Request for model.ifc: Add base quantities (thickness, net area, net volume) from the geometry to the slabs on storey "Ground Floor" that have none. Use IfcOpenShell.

First a look at what the model holds.

```python
import ifcopenshell
import ifcopenshell.util.element
import ifcopenshell.util.unit

model = ifcopenshell.open("model.ifc")
print(model.schema)
for unit_type in ("LENGTHUNIT", "AREAUNIT", "VOLUMEUNIT"):
    print(unit_type, ifcopenshell.util.unit.calculate_unit_scale(model, unit_type))
storey = next(s for s in model.by_type("IfcBuildingStorey") if s.Name == "Ground Floor")
slabs = [e for e in ifcopenshell.util.element.get_decomposition(storey) if e.is_a("IfcSlab")]
for e in sorted(slabs, key=lambda e: e.id()):
    print(e.id(), e.is_a(), e.Name, list(ifcopenshell.util.element.get_psets(e, qtos_only=True)), sep=" | ")
```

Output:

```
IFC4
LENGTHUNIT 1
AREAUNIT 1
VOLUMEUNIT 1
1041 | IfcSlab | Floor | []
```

```python
import ifcopenshell
import ifcopenshell.api.pset
import ifcopenshell.geom
import ifcopenshell.util.element
import ifcopenshell.util.shape
import ifcopenshell.util.unit

model = ifcopenshell.open("model.ifc")
unit_scale = ifcopenshell.util.unit.calculate_unit_scale(model)
area_scale = ifcopenshell.util.unit.calculate_unit_scale(model, "AREAUNIT")
volume_scale = ifcopenshell.util.unit.calculate_unit_scale(model, "VOLUMEUNIT")
settings = ifcopenshell.geom.settings()

storey = next(s for s in model.by_type("IfcBuildingStorey") if s.Name == "Ground Floor")
slabs = [e for e in ifcopenshell.util.element.get_decomposition(storey) if e.is_a("IfcSlab")]

for e in sorted(slabs, key=lambda e: e.id()):
    if ifcopenshell.util.element.get_psets(e, qtos_only=True, should_inherit=False):
        continue
    # Geometry comes back in metres, in the element's own axes.
    shape = ifcopenshell.geom.create_shape(settings, e)
    values = {
        "Width": ifcopenshell.util.shape.get_z(shape.geometry) / unit_scale,
        "NetArea": ifcopenshell.util.shape.get_footprint_area(shape.geometry) / area_scale,
        "NetVolume": ifcopenshell.util.shape.get_volume(shape.geometry) / volume_scale,
    }
    qto = ifcopenshell.api.pset.add_qto(model, product=e, name="Qto_SlabBaseQuantities")
    ifcopenshell.api.pset.edit_qto(model, qto=qto, properties=values)
    print(e.id(), {k: round(v, 3) for k, v in values.items()})

model.write("model_updated.ifc")
```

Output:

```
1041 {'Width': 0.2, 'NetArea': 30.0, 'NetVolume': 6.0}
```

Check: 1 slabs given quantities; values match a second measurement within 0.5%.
